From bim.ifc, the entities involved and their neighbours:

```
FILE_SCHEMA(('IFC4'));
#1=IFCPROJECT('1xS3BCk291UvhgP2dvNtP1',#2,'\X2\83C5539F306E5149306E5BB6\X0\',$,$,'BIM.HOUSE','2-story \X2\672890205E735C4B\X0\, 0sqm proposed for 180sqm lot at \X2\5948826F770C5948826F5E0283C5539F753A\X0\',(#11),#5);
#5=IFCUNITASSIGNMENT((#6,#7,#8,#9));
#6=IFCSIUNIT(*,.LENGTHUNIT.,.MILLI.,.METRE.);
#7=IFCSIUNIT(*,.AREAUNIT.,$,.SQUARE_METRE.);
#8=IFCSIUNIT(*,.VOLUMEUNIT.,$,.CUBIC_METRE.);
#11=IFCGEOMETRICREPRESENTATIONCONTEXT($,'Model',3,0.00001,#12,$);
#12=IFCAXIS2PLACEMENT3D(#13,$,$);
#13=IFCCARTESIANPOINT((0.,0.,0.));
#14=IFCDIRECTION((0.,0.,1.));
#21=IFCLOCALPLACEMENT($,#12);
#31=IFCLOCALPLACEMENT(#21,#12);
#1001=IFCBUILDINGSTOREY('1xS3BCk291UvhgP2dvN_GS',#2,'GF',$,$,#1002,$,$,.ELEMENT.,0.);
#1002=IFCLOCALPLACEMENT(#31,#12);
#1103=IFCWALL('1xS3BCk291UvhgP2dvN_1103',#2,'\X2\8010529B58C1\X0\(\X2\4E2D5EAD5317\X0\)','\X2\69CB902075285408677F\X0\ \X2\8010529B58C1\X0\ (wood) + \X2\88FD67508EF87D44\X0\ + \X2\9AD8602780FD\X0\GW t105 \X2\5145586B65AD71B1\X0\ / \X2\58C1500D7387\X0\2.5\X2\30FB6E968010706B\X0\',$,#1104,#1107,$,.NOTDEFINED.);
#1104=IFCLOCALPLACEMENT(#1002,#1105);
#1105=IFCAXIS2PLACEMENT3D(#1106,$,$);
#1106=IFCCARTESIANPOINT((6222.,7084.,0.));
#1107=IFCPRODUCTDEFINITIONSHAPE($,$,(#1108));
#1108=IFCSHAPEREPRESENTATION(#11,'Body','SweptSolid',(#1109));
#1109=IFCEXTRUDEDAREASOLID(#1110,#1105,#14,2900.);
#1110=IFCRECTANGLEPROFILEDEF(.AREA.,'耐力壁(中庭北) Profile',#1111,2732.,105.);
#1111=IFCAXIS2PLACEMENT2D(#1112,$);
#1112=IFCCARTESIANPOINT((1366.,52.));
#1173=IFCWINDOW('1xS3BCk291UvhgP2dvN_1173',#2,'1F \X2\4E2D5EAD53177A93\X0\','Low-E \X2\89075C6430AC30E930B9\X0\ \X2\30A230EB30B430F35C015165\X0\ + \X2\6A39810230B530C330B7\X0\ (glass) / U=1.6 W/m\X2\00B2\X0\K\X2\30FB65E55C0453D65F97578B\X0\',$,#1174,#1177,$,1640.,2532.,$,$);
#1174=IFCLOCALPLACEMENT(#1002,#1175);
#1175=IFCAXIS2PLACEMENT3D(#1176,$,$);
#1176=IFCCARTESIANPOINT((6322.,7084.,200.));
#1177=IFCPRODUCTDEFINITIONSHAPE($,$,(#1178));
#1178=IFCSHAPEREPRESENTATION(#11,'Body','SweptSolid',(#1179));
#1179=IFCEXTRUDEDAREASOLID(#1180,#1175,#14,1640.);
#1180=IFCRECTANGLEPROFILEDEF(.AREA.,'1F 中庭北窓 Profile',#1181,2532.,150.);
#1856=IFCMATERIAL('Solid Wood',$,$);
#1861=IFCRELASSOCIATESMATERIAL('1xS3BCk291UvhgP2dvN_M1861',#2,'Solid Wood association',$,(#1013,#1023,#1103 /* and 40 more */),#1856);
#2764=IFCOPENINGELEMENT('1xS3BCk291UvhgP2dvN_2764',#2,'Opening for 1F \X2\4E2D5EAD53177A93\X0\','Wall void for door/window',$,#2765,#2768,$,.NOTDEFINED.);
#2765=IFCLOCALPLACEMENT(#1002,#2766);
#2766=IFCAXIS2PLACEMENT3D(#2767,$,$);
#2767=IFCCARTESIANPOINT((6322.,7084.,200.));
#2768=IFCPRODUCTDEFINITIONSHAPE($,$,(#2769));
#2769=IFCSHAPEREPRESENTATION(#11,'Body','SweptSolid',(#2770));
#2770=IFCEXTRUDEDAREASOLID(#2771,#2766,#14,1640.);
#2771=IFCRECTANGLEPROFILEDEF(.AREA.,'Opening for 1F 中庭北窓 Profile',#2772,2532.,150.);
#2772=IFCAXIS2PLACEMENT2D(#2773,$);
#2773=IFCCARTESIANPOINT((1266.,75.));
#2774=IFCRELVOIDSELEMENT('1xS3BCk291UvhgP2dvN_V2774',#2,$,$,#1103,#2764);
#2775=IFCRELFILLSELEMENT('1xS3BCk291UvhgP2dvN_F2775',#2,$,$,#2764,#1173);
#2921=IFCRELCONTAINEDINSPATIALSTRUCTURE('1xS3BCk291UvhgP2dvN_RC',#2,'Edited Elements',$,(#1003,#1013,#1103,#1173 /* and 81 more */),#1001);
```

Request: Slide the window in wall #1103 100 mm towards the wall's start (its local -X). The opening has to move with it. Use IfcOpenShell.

```python
import ifcopenshell
import ifcopenshell.api.geometry
import ifcopenshell.util.placement

model = ifcopenshell.open("bim.ifc")

window = model.by_guid("1xS3BCk291UvhgP2dvN_1173")
opening = window.FillsVoids[0].RelatingOpeningElement
wall = opening.VoidsElements[0].RelatingBuildingElement

wall_matrix = ifcopenshell.util.placement.get_local_placement(wall.ObjectPlacement)
shift = wall_matrix[:3, 0] * -100.0
before = ifcopenshell.util.placement.get_local_placement(window.ObjectPlacement)[:3, 3].copy()

# The window is not placed relative to its opening, so move both.
for product in (opening, window):
    matrix = ifcopenshell.util.placement.get_local_placement(product.ObjectPlacement)
    matrix[:3, 3] += shift
    ifcopenshell.api.geometry.edit_object_placement(model, product=product, matrix=matrix, is_si=False)

after = ifcopenshell.util.placement.get_local_placement(window.ObjectPlacement)[:3, 3]
print("window moved by", (after - before).round(3) + 0.0)

model.write("bim_updated.ifc")
```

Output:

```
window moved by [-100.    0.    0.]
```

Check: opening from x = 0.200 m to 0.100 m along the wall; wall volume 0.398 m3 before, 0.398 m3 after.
